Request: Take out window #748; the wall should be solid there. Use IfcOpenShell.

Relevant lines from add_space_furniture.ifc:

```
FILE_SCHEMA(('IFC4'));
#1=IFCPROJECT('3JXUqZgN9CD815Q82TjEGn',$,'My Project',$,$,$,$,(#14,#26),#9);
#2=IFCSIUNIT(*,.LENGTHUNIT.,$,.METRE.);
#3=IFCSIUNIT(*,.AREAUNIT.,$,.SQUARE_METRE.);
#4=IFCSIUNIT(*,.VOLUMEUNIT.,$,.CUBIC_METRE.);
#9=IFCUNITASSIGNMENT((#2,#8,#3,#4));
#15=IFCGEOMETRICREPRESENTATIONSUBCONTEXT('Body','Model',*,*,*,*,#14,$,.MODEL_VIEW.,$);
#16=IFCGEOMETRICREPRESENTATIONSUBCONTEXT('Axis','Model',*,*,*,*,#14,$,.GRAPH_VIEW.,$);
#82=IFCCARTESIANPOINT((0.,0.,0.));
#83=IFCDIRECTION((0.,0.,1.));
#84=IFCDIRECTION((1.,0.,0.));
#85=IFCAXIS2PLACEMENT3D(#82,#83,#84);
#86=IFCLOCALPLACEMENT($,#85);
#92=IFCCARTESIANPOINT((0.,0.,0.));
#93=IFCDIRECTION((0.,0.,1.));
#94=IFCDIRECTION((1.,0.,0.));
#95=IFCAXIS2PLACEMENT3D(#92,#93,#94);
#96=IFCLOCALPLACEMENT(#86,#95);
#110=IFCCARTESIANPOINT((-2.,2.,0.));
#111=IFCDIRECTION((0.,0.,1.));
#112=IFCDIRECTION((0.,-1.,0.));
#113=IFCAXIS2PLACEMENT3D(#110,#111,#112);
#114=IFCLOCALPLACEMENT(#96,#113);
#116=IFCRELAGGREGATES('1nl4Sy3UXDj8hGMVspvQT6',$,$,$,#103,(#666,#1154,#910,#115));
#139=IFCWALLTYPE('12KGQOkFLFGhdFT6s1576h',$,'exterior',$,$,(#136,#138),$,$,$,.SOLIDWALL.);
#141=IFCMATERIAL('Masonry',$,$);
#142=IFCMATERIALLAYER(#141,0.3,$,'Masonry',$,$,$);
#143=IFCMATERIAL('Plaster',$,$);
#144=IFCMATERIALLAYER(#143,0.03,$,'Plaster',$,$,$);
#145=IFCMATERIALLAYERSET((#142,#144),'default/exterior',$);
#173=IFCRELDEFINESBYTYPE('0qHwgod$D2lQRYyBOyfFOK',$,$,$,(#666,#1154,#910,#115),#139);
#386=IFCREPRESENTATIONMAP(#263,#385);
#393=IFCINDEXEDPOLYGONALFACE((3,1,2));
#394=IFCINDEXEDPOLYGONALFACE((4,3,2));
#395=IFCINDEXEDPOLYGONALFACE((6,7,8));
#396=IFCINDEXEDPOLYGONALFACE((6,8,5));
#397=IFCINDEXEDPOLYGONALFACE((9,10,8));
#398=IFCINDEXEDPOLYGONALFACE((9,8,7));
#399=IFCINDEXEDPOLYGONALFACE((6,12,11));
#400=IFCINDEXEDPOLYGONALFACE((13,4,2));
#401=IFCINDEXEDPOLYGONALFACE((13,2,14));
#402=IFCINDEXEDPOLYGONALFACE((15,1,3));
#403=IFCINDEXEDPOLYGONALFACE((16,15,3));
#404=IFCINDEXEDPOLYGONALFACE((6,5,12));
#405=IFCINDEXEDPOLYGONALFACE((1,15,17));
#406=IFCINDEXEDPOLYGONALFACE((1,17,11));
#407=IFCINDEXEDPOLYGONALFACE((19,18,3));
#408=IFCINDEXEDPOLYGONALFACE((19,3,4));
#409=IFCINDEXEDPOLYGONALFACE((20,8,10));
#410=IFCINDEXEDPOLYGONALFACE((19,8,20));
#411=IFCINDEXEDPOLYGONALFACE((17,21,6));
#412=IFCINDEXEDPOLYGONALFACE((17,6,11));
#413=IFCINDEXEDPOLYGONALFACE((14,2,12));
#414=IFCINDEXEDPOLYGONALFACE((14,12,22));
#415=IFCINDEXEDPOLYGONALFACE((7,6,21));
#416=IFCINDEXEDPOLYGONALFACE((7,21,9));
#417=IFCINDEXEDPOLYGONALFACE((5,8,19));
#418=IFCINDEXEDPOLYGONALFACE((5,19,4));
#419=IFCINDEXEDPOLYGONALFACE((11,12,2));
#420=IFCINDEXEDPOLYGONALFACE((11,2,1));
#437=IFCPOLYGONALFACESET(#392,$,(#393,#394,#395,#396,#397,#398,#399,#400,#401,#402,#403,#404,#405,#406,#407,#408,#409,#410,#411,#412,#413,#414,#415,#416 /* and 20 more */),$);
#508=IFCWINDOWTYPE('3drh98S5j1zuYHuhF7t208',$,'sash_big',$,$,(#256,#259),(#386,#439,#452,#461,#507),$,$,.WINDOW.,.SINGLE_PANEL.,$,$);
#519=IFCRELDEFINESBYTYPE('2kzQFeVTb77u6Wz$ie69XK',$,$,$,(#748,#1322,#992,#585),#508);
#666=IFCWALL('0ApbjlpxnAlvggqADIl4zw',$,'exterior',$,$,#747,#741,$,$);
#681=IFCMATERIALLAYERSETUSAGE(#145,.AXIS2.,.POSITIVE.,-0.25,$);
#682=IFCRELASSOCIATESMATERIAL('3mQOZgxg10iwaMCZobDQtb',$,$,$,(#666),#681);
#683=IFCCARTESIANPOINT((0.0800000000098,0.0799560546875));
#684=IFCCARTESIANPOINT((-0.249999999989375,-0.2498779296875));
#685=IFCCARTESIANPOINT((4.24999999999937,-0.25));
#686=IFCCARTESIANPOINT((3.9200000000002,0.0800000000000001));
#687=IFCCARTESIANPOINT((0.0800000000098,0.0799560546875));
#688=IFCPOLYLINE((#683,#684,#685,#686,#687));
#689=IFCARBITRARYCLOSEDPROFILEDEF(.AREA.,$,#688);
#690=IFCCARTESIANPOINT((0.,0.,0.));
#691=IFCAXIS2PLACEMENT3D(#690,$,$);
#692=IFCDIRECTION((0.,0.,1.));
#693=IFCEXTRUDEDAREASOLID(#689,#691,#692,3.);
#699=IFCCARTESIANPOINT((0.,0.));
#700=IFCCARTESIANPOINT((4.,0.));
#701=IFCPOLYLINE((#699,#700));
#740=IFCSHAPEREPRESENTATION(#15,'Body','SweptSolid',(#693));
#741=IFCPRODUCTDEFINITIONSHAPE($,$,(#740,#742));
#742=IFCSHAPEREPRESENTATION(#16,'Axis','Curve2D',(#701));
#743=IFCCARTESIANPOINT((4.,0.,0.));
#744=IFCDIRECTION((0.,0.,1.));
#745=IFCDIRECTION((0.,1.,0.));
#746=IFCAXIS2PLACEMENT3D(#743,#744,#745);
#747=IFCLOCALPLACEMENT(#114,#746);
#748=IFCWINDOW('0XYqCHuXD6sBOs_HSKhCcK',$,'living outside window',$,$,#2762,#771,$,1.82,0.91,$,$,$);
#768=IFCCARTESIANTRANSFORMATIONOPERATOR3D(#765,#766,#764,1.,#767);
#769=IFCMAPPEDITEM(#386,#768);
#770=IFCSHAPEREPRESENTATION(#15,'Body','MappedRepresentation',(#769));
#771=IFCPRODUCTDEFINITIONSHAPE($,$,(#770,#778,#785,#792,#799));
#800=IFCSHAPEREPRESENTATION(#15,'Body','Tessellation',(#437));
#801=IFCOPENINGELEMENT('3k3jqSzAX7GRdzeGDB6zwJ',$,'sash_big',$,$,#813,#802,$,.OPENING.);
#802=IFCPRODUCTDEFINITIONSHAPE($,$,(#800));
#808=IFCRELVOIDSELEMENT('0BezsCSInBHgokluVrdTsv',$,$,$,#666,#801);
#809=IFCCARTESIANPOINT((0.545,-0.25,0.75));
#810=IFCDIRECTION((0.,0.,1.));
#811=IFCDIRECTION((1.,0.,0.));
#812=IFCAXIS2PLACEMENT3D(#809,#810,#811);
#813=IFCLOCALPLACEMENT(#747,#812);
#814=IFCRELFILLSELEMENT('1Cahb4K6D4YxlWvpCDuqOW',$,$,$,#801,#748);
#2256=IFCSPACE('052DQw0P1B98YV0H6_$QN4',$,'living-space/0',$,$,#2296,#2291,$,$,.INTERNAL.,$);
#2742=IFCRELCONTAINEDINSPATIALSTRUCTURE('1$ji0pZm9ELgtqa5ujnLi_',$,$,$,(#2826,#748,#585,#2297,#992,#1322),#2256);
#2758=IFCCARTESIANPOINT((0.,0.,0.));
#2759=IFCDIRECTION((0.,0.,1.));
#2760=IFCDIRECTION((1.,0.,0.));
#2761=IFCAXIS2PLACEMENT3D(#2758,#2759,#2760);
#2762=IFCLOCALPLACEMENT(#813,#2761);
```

```python
import ifcopenshell
import ifcopenshell.api.feature
import ifcopenshell.api.root
import ifcopenshell.geom
import ifcopenshell.util.shape

model = ifcopenshell.open("add_space_furniture.ifc")
settings = ifcopenshell.geom.settings()


def volume(element):
    """Net volume in cubic metres, openings subtracted."""
    shape = ifcopenshell.geom.create_shape(settings, element)
    return ifcopenshell.util.shape.get_volume(shape.geometry)


window = model.by_guid("0XYqCHuXD6sBOs_HSKhCcK")
opening = window.FillsVoids[0].RelatingOpeningElement
wall = opening.VoidsElements[0].RelatingBuildingElement
before = volume(wall)

ifcopenshell.api.root.remove_product(model, product=window)
ifcopenshell.api.feature.remove_feature(model, feature=opening)

after = volume(wall)

print(f"wall volume {before:.3f} -> {after:.3f} m3")

model.write("add_space_furniture_updated.ifc")
```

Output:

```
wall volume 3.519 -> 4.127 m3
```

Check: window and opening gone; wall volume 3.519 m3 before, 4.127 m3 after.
